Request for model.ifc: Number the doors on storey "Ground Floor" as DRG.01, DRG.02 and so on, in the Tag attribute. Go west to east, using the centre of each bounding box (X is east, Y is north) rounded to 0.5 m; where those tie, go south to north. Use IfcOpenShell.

First a look at what the model holds.

```python
import ifcopenshell
import ifcopenshell.util.element
import ifcopenshell.util.placement

model = ifcopenshell.open("model.ifc")
print(model.schema)
storey = next(s for s in model.by_type("IfcBuildingStorey") if s.Name == "Ground Floor")
doors = [e for e in ifcopenshell.util.element.get_decomposition(storey) if e.is_a("IfcDoor")]
for e in sorted(doors, key=lambda e: e.id()):
    origin = ifcopenshell.util.placement.get_local_placement(e.ObjectPlacement)[:3, 3]
    print(e.id(), e.Tag, e.Name, origin.round(2) + 0.0, sep=" | ")
```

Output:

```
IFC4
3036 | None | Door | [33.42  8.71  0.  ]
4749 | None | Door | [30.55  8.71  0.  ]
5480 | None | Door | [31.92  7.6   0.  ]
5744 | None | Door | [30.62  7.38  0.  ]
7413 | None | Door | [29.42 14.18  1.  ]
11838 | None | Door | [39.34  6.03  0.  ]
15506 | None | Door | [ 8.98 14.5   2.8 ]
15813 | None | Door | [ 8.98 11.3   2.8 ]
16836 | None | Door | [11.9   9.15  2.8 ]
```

```python
import ifcopenshell
import ifcopenshell.geom
import ifcopenshell.util.element
import ifcopenshell.util.shape

model = ifcopenshell.open("model.ifc")
settings = ifcopenshell.geom.settings()
settings.set("use-world-coords", True)


def centre(element):
    shape = ifcopenshell.geom.create_shape(settings, element)
    return ifcopenshell.util.shape.get_bbox_centroid(shape.geometry)


storey = next(s for s in model.by_type("IfcBuildingStorey") if s.Name == "Ground Floor")
doors = [e for e in ifcopenshell.util.element.get_decomposition(storey) if e.is_a("IfcDoor")]

# Insertion points can sit at a corner or the storey origin, so sort by the geometry (in metres).
centres = {e: centre(e) for e in doors}
doors.sort(key=lambda e: (round(centres[e][0] / 0.5), centres[e][1]))

for i, e in enumerate(doors, start=1):
    number = f"DRG.{i:02d}"
    e.Tag = number
    print(e.id(), number)

model.write("model_rev.ifc")
```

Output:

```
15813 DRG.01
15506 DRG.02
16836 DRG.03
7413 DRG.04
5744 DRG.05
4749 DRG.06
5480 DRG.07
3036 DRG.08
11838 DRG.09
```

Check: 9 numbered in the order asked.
